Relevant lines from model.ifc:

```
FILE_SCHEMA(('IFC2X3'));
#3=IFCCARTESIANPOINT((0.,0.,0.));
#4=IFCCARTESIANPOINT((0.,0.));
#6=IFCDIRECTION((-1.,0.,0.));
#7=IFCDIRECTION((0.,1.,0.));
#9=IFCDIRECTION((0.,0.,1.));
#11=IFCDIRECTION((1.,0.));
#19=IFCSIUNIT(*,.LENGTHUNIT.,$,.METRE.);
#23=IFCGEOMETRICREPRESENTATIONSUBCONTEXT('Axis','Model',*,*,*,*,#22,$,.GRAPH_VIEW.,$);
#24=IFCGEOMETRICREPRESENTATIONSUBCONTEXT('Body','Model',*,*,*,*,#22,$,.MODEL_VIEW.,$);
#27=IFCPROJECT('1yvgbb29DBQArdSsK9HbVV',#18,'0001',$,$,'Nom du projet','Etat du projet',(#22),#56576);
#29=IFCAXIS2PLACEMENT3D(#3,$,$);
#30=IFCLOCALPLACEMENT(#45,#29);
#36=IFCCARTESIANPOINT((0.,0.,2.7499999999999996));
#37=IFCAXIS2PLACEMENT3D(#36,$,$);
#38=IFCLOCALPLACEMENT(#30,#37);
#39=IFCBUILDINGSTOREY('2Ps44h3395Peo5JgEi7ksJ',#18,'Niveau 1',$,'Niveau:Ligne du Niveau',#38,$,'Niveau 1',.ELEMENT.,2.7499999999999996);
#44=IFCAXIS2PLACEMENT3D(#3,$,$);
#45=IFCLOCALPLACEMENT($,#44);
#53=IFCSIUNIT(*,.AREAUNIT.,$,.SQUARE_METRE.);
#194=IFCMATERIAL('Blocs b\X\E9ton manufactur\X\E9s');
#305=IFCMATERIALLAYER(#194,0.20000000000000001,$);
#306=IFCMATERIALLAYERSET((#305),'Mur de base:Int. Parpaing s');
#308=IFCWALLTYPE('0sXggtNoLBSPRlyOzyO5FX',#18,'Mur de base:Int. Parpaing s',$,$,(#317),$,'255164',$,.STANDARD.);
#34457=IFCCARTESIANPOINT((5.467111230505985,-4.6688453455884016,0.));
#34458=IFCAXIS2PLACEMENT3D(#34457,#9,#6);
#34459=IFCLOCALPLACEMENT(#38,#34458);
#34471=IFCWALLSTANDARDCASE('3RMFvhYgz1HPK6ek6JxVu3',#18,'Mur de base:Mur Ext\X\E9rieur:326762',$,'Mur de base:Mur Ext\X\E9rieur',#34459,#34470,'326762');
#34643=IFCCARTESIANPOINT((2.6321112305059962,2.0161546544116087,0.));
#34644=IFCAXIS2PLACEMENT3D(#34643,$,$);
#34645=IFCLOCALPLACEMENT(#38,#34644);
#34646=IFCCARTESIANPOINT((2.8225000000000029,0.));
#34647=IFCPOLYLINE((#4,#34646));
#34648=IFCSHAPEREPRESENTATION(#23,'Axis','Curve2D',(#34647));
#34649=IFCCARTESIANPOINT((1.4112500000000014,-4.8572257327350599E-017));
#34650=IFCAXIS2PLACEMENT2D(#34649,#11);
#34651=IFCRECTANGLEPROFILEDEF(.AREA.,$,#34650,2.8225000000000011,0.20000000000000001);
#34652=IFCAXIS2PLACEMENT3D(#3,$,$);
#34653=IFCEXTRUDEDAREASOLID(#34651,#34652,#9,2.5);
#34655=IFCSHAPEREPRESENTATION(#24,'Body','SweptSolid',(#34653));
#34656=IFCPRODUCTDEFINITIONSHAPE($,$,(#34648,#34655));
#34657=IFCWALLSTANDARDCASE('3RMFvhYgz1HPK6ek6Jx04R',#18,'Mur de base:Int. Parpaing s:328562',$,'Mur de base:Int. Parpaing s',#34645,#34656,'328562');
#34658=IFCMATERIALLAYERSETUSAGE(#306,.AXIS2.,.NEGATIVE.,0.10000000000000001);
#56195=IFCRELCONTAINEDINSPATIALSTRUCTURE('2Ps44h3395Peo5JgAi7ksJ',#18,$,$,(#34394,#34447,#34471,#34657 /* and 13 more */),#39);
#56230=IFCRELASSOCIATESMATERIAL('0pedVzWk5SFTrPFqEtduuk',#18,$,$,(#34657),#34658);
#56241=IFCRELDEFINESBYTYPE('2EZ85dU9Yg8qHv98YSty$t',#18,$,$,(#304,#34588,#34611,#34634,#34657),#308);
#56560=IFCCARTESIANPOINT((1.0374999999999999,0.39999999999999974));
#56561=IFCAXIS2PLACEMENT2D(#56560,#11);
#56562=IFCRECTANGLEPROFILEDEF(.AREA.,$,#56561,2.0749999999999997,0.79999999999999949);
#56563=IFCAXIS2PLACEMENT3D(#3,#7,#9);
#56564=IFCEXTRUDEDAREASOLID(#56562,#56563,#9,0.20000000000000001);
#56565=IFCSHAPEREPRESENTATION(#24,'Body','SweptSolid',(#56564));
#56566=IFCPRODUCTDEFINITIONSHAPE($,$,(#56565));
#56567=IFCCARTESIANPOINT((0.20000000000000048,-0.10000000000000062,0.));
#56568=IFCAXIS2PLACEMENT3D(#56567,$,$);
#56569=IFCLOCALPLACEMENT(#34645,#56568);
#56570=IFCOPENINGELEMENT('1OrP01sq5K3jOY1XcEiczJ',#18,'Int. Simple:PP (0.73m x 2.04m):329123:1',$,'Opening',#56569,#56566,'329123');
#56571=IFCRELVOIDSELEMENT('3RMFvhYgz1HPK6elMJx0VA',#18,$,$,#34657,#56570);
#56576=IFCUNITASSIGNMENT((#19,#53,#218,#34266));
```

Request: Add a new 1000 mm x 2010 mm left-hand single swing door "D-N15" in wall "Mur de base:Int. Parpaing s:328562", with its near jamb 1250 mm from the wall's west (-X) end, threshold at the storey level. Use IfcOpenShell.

```python
import numpy as np
import ifcopenshell
import ifcopenshell.api.feature
import ifcopenshell.api.geometry
import ifcopenshell.api.root
import ifcopenshell.api.spatial
import ifcopenshell.api.type
import ifcopenshell.geom
import ifcopenshell.util.element
import ifcopenshell.util.placement
import ifcopenshell.util.representation
import ifcopenshell.util.shape
import ifcopenshell.util.unit

model = ifcopenshell.open("model.ifc")
unit_scale = ifcopenshell.util.unit.calculate_unit_scale(model)
settings = ifcopenshell.geom.settings()


def volume(element):
    """Net volume in cubic metres, openings subtracted."""
    shape = ifcopenshell.geom.create_shape(settings, element)
    return ifcopenshell.util.shape.get_volume(shape.geometry)


wall = model.by_guid("3RMFvhYgz1HPK6ek6Jx04R")
storey = ifcopenshell.util.element.get_container(wall, ifc_class="IfcBuildingStorey")
context = ifcopenshell.util.representation.get_context(model, "Model", "Body", "MODEL_VIEW")
before = volume(wall)

width, height, from_end, sill = 1, 2.01, 1.25, 0.0  # metres

# The wall runs along its own X axis, and the end named is its -X end.
wall_shape = ifcopenshell.geom.create_shape(settings, wall)
x, y, z = ifcopenshell.util.shape.get_vertices(wall_shape.geometry).T
start = x.min() + from_end
face, thickness = float(y.min()), float(y.max() - y.min())
wall_matrix = ifcopenshell.util.placement.get_local_placement(wall.ObjectPlacement)
level = ifcopenshell.util.placement.get_local_placement(storey.ObjectPlacement)[2, 3]


def in_wall(x, y):
    """Placement at x, y metres in the wall's axes, at sill height."""
    matrix = wall_matrix.copy()
    matrix[:, 3] = wall_matrix @ np.array([x / unit_scale, y / unit_scale, 0.0, 1.0])
    matrix[2, 3] = level + sill / unit_scale
    return matrix


# Opening: a box that overshoots both wall faces by 50 mm.
opening = ifcopenshell.api.root.create_entity(model, ifc_class="IfcOpeningElement")
box = ifcopenshell.api.geometry.add_wall_representation(
    model, context=context, length=width, height=height, thickness=thickness + 0.1
)
ifcopenshell.api.geometry.assign_representation(model, product=opening, representation=box)
ifcopenshell.api.geometry.edit_object_placement(model, product=opening, matrix=in_wall(start, face - 0.05), is_si=False)
ifcopenshell.api.feature.add_feature(model, feature=opening, element=wall)

door = ifcopenshell.api.root.create_entity(model, ifc_class="IfcDoor", name="D-N15")
door.OverallWidth, door.OverallHeight = width / unit_scale, height / unit_scale
body = ifcopenshell.api.geometry.add_door_representation(
    model,
    context=context,
    overall_width=door.OverallWidth,
    overall_height=door.OverallHeight,
    operation_type="SINGLE_SWING_LEFT",
    lining_properties={"LiningDepth": thickness / unit_scale, "ThresholdDepth": thickness / unit_scale},
)
ifcopenshell.api.geometry.assign_representation(model, product=door, representation=body)
ifcopenshell.api.spatial.assign_container(model, products=[door], relating_structure=storey)
fills = ifcopenshell.api.feature.add_filling(model, opening=opening, element=door)
fills.OwnerHistory = door.OwnerHistory  # required in IFC2X3

# IFC2X3 keeps the operation on the door style.
style = ifcopenshell.api.root.create_entity(model, ifc_class="IfcDoorStyle", name="D-N15")
style.OperationType, style.ConstructionType = "SINGLE_SWING_LEFT", "NOTDEFINED"
style.ParameterTakesPrecedence = style.Sizeable = False
ifcopenshell.api.type.assign_type(model, related_objects=[door], relating_type=style)

# The lining spans the wall, so the door starts at the wall face.
ifcopenshell.api.geometry.edit_object_placement(model, product=door, matrix=in_wall(start, face), is_si=False)

after = volume(wall)

print(f"wall volume {before:.3f} -> {after:.3f} m3")

model.write("model_updated.ifc")
```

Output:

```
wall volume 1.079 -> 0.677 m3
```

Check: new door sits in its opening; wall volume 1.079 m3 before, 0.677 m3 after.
